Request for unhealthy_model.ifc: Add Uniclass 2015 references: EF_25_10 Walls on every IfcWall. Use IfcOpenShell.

First a look at what the model holds.

```python
import ifcopenshell

model = ifcopenshell.open("unhealthy_model.ifc")
print(model.schema)
print("classifications:", [c.Name for c in model.by_type("IfcClassification")])
for ifc_class in ("IfcDoor", "IfcRoof", "IfcStair", "IfcWall", "IfcWindow"):
    print(ifc_class, len(model.by_type(ifc_class)))
```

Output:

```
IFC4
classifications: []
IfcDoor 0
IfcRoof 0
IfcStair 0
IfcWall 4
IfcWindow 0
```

```python
import ifcopenshell
import ifcopenshell.api.classification

model = ifcopenshell.open("unhealthy_model.ifc")

system = ifcopenshell.api.classification.add_classification(model, classification="Uniclass 2015")

codes = {
    "IfcWall": ("EF_25_10", "Walls"),
}
for ifc_class, (code, name) in codes.items():
    products = model.by_type(ifc_class)
    ifcopenshell.api.classification.add_reference(
        model, products=products, classification=system, identification=code, name=name
    )
    print(code, len(products))

model.write("unhealthy_model_rev.ifc")
```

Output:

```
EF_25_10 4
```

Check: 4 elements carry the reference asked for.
